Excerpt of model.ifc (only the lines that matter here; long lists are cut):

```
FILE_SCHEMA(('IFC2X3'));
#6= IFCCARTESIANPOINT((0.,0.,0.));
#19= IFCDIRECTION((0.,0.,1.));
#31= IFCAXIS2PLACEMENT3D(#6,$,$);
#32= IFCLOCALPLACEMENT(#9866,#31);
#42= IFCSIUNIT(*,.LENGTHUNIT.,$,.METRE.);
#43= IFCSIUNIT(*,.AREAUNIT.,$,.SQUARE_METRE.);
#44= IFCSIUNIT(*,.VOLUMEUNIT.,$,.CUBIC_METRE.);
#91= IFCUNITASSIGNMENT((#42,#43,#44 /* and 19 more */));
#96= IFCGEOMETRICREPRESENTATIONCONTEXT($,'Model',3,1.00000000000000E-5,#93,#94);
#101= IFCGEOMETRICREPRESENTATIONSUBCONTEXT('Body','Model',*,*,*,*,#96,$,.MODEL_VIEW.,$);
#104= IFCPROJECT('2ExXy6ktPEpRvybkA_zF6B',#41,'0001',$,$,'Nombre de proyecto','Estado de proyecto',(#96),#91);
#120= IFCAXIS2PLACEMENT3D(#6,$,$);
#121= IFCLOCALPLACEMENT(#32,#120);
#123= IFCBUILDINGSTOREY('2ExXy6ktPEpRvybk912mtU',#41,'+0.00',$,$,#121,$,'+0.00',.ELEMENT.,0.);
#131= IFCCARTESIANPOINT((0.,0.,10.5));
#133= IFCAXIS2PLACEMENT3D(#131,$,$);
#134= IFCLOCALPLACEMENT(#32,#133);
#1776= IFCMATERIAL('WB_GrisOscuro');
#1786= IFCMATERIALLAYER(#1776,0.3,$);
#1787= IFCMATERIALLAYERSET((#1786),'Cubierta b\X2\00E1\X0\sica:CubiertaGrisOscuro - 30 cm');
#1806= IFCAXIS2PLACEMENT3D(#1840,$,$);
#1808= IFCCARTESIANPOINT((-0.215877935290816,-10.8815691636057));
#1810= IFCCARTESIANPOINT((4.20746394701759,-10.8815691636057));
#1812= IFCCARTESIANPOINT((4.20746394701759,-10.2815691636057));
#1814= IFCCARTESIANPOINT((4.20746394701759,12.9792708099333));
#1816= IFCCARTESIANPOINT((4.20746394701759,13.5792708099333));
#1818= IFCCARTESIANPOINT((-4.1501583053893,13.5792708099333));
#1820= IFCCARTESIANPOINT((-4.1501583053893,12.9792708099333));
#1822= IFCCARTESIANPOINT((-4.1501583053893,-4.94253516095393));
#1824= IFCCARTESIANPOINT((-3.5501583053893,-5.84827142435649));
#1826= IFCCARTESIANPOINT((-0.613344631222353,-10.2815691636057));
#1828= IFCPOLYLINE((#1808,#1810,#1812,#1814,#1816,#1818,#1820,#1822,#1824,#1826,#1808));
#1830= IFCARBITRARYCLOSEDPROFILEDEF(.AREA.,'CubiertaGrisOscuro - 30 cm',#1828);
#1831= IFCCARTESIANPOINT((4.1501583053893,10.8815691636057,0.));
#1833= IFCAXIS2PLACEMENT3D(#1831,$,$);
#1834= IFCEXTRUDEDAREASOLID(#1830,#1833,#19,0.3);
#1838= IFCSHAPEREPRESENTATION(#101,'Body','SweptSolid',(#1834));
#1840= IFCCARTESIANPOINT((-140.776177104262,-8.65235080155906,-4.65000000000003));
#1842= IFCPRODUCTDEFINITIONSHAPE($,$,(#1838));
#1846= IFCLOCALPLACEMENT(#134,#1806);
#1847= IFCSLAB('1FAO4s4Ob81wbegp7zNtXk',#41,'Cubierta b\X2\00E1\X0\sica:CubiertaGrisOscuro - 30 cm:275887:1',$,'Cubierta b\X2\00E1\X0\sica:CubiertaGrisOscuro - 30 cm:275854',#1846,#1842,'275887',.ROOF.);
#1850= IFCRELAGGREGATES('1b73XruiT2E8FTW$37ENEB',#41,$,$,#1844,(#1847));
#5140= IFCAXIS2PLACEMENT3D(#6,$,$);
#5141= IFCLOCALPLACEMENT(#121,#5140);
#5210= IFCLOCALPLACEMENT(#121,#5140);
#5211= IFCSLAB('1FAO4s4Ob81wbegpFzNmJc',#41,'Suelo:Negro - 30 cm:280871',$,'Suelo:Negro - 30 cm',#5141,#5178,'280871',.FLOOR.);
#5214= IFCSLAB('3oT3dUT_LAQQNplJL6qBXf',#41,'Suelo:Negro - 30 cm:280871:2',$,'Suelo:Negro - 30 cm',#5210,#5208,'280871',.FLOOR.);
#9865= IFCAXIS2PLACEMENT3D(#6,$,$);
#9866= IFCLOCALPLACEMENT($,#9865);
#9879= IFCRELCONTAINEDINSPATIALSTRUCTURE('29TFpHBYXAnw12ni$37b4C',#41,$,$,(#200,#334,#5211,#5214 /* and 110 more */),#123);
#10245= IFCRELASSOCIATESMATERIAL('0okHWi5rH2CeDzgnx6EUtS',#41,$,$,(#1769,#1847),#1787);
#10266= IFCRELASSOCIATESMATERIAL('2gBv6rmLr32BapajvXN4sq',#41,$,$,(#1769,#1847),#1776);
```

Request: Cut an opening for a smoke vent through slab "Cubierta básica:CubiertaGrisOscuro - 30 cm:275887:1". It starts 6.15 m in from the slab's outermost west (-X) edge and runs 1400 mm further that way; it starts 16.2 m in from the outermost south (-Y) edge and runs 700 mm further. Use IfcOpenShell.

```python
import numpy as np
import ifcopenshell
import ifcopenshell.api.feature
import ifcopenshell.api.geometry
import ifcopenshell.api.root
import ifcopenshell.geom
import ifcopenshell.util.placement
import ifcopenshell.util.representation
import ifcopenshell.util.shape
import ifcopenshell.util.unit

model = ifcopenshell.open("model.ifc")
unit_scale = ifcopenshell.util.unit.calculate_unit_scale(model)
settings = ifcopenshell.geom.settings()


def volume(element):
    """Net volume in cubic metres, openings subtracted."""
    shape = ifcopenshell.geom.create_shape(settings, element)
    return ifcopenshell.util.shape.get_volume(shape.geometry)


slab = model.by_guid("1FAO4s4Ob81wbegp7zNtXk")
before = volume(slab)

# Extent in the slab's own axes, in metres. The edges named are its -X and -Y sides.
slab_shape = ifcopenshell.geom.create_shape(settings, slab)
vertices = ifcopenshell.util.shape.get_vertices(slab_shape.geometry)
x_min, y_min, bottom = vertices.min(axis=0)
top = vertices[:, 2].max()

opening = ifcopenshell.api.root.create_entity(model, ifc_class="IfcOpeningElement", name="Smoke vent opening")
context = ifcopenshell.util.representation.get_context(model, "Model", "Body", "MODEL_VIEW")
width, depth = 1.4, 0.7
outline = [(0.0, 0.0), (width, 0.0), (width, depth), (0.0, depth), (0.0, 0.0)]
# Overshoot both faces by 50 mm so the cut is clean.
shape = ifcopenshell.api.geometry.add_slab_representation(
    model, context=context, depth=top - bottom + 0.1, polyline=outline
)
ifcopenshell.api.geometry.assign_representation(model, product=opening, representation=shape)

matrix = ifcopenshell.util.placement.get_local_placement(slab.ObjectPlacement)
matrix[:, 3] = matrix @ np.append(np.array([x_min + 6.15, y_min + 16.2, bottom - 0.05]) / unit_scale, 1.0)
ifcopenshell.api.geometry.edit_object_placement(model, product=opening, matrix=matrix, is_si=False)
ifcopenshell.api.feature.add_feature(model, feature=opening, element=slab)

after = volume(slab)

print(f"slab volume {before:.3f} -> {after:.3f} m3")

model.write("model_v2.ifc")
```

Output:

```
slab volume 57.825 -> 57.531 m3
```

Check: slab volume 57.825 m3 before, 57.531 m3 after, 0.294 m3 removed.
